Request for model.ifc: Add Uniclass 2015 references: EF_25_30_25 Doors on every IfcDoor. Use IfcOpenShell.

First a look at what the model holds.

```python
import ifcopenshell

model = ifcopenshell.open("model.ifc")
print(model.schema)
print("classifications:", [c.Name for c in model.by_type("IfcClassification")])
for ifc_class in ("IfcDoor", "IfcRoof", "IfcStair", "IfcWall", "IfcWindow"):
    print(ifc_class, len(model.by_type(ifc_class)))
```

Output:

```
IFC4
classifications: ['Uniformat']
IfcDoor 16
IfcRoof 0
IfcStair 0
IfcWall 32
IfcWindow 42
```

```python
import ifcopenshell
import ifcopenshell.api.classification

model = ifcopenshell.open("model.ifc")

system = ifcopenshell.api.classification.add_classification(model, classification="Uniclass 2015")

codes = {
    "IfcDoor": ("EF_25_30_25", "Doors"),
}
for ifc_class, (code, name) in codes.items():
    products = model.by_type(ifc_class)
    ifcopenshell.api.classification.add_reference(
        model, products=products, classification=system, identification=code, name=name
    )
    print(code, len(products))

model.write("model_updated.ifc")
```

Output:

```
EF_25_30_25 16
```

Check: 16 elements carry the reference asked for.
